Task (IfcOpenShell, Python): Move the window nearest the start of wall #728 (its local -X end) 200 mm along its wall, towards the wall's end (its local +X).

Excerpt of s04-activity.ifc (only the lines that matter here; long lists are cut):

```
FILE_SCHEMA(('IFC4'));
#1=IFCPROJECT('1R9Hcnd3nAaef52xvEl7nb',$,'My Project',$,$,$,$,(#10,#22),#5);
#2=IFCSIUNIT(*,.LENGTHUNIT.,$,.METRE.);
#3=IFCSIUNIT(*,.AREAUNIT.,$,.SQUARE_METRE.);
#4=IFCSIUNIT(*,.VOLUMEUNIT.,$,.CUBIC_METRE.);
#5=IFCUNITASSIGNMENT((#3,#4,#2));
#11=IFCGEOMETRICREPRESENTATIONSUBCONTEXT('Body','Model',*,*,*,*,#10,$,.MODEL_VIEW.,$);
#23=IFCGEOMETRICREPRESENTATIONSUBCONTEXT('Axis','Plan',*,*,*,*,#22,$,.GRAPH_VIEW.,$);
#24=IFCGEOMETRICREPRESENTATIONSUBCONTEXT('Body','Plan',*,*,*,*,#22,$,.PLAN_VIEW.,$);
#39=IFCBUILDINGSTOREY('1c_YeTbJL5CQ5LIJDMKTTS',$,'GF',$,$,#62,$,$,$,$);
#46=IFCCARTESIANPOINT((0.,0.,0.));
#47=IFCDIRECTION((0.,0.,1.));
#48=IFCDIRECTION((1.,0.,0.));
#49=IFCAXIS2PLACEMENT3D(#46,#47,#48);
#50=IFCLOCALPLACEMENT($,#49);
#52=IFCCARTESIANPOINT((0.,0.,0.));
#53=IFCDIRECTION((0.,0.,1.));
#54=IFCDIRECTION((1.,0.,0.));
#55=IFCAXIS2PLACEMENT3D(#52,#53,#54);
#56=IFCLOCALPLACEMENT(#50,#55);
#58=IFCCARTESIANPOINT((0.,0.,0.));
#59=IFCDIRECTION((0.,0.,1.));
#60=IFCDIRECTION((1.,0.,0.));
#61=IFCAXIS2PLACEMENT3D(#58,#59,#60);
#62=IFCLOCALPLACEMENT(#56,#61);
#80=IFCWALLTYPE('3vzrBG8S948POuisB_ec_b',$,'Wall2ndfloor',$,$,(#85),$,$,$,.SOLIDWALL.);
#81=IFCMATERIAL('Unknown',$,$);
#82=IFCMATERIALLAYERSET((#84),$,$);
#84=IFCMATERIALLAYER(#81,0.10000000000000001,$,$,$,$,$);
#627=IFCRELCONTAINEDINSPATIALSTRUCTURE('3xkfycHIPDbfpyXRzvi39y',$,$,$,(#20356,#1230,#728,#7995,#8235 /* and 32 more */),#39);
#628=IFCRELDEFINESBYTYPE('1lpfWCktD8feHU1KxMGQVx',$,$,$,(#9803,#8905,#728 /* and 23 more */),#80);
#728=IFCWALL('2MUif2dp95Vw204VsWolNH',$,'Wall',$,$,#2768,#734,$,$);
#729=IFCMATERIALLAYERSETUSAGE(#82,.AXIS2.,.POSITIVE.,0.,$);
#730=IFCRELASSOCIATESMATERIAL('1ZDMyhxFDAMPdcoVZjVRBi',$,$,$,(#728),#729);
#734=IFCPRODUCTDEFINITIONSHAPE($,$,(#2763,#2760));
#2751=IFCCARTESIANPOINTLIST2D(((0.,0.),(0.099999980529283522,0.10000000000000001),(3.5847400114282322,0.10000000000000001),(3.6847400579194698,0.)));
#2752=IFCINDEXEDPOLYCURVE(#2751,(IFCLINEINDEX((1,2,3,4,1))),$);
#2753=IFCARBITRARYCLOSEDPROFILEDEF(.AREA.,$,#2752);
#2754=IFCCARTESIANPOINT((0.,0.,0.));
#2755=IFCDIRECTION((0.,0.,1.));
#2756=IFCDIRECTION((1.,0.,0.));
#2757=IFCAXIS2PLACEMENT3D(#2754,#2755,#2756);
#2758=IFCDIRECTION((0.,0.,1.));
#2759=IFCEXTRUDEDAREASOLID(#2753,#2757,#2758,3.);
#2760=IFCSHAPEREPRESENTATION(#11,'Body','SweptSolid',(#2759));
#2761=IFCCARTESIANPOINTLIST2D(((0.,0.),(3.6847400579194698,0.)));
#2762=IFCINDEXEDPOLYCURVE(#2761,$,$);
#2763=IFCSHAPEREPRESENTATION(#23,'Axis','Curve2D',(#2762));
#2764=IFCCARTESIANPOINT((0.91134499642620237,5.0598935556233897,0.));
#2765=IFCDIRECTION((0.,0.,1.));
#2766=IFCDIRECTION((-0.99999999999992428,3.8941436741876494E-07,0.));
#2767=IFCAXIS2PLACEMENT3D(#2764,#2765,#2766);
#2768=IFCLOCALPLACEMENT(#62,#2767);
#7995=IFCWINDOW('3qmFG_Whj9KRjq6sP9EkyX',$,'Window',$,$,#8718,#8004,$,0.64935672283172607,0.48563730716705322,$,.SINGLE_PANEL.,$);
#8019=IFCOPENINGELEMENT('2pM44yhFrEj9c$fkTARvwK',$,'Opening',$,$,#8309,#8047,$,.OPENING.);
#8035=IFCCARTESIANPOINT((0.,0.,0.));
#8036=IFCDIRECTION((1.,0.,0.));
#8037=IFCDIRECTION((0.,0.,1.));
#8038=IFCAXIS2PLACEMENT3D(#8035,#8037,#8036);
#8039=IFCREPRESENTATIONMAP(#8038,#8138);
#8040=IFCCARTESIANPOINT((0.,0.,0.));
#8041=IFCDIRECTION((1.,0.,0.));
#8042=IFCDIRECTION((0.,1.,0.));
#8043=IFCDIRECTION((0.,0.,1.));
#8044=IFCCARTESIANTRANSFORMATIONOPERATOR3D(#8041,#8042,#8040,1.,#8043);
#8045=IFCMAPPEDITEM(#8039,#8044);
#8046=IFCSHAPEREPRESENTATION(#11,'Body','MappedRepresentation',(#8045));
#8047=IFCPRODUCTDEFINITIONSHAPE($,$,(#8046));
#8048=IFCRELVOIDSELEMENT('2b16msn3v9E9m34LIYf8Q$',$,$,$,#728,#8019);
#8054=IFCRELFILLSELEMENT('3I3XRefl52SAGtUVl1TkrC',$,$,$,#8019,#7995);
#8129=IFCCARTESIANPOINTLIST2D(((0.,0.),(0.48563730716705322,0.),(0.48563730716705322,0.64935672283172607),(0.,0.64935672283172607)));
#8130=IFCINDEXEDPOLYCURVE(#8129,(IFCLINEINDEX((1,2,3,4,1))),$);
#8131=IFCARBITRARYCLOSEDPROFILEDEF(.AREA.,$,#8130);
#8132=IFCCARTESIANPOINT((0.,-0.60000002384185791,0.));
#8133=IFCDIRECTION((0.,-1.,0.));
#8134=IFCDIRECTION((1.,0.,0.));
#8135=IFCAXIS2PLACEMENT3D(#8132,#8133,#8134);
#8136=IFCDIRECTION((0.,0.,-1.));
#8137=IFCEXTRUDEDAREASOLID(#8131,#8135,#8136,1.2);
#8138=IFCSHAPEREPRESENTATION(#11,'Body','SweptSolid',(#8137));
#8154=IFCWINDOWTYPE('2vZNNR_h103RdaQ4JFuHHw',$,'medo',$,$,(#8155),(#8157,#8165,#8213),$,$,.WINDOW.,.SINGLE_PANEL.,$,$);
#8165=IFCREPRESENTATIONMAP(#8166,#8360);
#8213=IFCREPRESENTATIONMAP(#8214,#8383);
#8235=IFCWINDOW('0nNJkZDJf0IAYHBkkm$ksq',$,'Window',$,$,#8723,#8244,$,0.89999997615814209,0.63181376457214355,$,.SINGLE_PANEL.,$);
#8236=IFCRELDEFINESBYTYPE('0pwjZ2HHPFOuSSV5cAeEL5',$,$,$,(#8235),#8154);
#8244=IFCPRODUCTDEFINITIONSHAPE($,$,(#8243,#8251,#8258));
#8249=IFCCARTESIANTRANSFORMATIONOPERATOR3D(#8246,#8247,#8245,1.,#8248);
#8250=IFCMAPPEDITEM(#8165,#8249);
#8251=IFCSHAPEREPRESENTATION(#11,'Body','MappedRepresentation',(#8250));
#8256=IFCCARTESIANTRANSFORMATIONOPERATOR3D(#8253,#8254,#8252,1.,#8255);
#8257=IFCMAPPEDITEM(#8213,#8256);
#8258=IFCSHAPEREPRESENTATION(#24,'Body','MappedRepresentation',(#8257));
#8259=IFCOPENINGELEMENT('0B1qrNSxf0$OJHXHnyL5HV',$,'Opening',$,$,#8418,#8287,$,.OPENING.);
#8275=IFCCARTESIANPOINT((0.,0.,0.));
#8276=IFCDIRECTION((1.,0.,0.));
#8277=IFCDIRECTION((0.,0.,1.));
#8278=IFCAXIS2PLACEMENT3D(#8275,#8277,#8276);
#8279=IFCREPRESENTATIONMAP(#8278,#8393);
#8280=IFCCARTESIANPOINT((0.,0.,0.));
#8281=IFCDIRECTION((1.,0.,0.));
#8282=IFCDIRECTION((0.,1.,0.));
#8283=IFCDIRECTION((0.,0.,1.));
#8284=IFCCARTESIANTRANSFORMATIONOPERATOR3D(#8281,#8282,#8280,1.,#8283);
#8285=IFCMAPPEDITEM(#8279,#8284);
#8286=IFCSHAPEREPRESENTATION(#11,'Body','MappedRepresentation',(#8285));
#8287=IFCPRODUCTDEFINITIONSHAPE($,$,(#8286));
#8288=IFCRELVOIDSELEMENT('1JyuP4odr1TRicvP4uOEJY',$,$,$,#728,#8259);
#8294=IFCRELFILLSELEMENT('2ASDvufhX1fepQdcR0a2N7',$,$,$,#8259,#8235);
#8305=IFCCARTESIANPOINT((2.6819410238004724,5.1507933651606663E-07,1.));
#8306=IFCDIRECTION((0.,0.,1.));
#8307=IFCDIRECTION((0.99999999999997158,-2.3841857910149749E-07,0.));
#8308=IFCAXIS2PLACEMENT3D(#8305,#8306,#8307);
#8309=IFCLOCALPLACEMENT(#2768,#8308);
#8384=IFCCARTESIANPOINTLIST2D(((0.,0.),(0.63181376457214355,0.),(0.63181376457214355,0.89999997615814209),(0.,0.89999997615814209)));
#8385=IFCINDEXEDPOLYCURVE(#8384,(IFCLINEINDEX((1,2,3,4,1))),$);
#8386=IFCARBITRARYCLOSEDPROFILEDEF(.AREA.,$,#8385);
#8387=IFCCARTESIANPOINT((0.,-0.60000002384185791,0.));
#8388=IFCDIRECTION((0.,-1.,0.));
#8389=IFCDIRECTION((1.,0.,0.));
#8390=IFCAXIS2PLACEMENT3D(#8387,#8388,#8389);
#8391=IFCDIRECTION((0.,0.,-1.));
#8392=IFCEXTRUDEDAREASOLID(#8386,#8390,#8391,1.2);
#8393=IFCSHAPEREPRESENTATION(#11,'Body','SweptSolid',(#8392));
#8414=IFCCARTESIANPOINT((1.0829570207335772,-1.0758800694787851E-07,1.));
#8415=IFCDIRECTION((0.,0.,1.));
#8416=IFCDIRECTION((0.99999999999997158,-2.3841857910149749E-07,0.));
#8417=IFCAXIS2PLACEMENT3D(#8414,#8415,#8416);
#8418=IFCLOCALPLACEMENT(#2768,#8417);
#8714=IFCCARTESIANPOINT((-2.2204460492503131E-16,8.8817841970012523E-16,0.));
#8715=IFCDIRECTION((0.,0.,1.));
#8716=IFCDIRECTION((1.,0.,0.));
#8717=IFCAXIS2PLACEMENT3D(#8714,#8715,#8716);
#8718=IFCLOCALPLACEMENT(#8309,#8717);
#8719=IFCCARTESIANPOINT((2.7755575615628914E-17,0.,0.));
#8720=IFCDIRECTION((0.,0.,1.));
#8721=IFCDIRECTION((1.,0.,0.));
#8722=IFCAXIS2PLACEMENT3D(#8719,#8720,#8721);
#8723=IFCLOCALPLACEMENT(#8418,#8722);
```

```python
import ifcopenshell
import ifcopenshell.api.geometry
import ifcopenshell.util.placement
import ifcopenshell.util.unit

model = ifcopenshell.open("s04-activity.ifc")
unit_scale = ifcopenshell.util.unit.calculate_unit_scale(model)

window = model.by_id(8235)
opening = window.FillsVoids[0].RelatingOpeningElement
wall = opening.VoidsElements[0].RelatingBuildingElement

wall_matrix = ifcopenshell.util.placement.get_local_placement(wall.ObjectPlacement)
shift = wall_matrix[:3, 0] * 0.2 / unit_scale
before = ifcopenshell.util.placement.get_local_placement(window.ObjectPlacement)[:3, 3].copy()

# The window is placed relative to its opening, so it follows when the opening moves.
matrix = ifcopenshell.util.placement.get_local_placement(opening.ObjectPlacement)
matrix[:3, 3] += shift
ifcopenshell.api.geometry.edit_object_placement(
    model, product=opening, matrix=matrix, is_si=False, should_transform_children=True
)

after = ifcopenshell.util.placement.get_local_placement(window.ObjectPlacement)[:3, 3]
print("window moved by", (after - before).round(3) + 0.0)

model.write("s04-activity-out.ifc")
```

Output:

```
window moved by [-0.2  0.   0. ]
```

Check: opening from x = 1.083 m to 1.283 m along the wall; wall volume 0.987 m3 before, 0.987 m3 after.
